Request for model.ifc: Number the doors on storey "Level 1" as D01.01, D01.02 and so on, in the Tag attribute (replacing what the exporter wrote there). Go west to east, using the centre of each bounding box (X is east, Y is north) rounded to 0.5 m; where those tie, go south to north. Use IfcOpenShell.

First a look at what the model holds.

```python
import ifcopenshell
import ifcopenshell.util.element
import ifcopenshell.util.placement

model = ifcopenshell.open("model.ifc")
print(model.schema)
storey = next(s for s in model.by_type("IfcBuildingStorey") if s.Name == "Level 1")
doors = [e for e in ifcopenshell.util.element.get_decomposition(storey) if e.is_a("IfcDoor")]
for e in sorted(doors, key=lambda e: e.id()):
    origin = ifcopenshell.util.placement.get_local_placement(e.ObjectPlacement)[:3, 3]
    print(e.id(), e.Tag, e.Name, origin.round(2) + 0.0, sep=" | ")
```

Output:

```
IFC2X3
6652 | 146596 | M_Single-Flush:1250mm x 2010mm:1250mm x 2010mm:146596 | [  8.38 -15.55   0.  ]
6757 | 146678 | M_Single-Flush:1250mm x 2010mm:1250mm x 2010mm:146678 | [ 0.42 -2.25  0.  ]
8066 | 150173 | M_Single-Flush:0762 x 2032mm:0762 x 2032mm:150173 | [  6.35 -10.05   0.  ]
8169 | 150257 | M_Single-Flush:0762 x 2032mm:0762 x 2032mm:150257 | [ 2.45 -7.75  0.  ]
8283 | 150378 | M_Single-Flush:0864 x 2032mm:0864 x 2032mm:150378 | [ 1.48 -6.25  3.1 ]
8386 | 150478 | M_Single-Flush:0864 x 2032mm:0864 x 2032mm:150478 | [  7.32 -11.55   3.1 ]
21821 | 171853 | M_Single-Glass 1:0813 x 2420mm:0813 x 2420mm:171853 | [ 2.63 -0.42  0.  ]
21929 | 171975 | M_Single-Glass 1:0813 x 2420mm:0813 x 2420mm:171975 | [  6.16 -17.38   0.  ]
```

```python
import ifcopenshell
import ifcopenshell.geom
import ifcopenshell.util.element
import ifcopenshell.util.shape

model = ifcopenshell.open("model.ifc")
settings = ifcopenshell.geom.settings()
settings.set("use-world-coords", True)


def centre(element):
    shape = ifcopenshell.geom.create_shape(settings, element)
    return ifcopenshell.util.shape.get_bbox_centroid(shape.geometry)


storey = next(s for s in model.by_type("IfcBuildingStorey") if s.Name == "Level 1")
doors = [e for e in ifcopenshell.util.element.get_decomposition(storey) if e.is_a("IfcDoor")]

# Insertion points can sit at a corner or the storey origin, so sort by the geometry (in metres).
centres = {e: centre(e) for e in doors}
doors.sort(key=lambda e: (round(centres[e][0] / 0.5), centres[e][1]))

for i, e in enumerate(doors, start=1):
    number = f"D01.{i:02d}"
    e.Tag = number
    print(e.id(), number)

model.write("model_rev.ifc")
```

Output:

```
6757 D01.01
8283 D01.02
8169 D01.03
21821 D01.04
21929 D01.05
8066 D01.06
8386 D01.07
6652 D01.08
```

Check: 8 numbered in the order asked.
